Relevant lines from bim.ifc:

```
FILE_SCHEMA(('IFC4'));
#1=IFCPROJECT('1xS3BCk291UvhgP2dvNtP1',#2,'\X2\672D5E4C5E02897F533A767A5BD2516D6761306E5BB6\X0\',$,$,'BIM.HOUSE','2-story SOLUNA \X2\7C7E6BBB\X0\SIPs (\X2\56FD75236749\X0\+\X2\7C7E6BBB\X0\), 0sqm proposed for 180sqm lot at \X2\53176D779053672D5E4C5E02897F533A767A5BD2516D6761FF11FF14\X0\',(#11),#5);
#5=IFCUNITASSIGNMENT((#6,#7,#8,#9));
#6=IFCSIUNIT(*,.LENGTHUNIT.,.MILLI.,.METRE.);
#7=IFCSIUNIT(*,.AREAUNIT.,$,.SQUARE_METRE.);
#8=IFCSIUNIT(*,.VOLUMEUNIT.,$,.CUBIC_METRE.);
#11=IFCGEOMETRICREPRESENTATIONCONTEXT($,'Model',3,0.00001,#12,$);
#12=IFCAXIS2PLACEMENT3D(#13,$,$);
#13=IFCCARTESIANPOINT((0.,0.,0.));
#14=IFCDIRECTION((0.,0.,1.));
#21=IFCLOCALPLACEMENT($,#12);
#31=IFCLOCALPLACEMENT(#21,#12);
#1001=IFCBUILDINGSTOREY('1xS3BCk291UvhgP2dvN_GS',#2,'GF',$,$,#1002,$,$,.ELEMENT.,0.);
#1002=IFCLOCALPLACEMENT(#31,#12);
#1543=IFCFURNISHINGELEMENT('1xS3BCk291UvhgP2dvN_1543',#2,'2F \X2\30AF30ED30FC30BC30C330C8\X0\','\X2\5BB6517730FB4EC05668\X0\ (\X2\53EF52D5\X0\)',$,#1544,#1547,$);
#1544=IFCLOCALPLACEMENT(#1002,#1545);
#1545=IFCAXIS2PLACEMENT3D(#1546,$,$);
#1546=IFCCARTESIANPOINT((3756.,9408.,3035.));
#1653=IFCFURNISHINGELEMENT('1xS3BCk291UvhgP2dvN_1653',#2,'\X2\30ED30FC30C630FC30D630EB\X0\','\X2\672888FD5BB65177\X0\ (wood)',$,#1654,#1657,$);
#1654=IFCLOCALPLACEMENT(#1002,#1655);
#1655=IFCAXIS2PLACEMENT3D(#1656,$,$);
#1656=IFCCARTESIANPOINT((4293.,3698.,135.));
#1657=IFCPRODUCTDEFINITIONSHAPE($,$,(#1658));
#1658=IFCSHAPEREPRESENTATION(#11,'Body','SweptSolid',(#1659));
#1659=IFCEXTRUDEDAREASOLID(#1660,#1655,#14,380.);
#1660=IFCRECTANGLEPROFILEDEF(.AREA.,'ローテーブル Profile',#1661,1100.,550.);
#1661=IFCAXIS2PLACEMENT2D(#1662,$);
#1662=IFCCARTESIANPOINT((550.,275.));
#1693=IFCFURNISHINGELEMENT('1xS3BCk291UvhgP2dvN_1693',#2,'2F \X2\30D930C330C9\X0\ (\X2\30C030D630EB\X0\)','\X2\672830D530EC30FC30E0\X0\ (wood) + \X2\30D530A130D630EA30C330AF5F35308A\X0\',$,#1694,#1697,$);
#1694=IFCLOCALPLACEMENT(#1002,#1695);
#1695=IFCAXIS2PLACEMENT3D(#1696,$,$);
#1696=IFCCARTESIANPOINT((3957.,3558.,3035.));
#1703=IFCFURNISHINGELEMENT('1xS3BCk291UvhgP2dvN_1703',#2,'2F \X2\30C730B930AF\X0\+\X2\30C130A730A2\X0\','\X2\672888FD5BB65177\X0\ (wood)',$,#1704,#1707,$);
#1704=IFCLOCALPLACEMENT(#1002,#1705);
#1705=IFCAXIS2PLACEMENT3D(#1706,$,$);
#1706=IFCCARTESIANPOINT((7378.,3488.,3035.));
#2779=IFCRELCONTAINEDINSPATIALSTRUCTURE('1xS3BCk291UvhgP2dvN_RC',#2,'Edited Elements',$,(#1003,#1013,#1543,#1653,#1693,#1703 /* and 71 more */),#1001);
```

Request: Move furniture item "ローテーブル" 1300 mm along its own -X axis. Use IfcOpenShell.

```python
import ifcopenshell
import ifcopenshell.api.geometry
import ifcopenshell.util.placement
import ifcopenshell.util.unit

model = ifcopenshell.open("bim.ifc")
unit_scale = ifcopenshell.util.unit.calculate_unit_scale(model)

item = model.by_id(1653)
matrix = ifcopenshell.util.placement.get_local_placement(item.ObjectPlacement)
matrix[:3, 3] -= matrix[:3, 0] * 1.3 / unit_scale
ifcopenshell.api.geometry.edit_object_placement(model, product=item, matrix=matrix, is_si=False)

print(ifcopenshell.util.placement.get_local_placement(item.ObjectPlacement).round(3) + 0.0)

model.write("bim_updated.ifc")
```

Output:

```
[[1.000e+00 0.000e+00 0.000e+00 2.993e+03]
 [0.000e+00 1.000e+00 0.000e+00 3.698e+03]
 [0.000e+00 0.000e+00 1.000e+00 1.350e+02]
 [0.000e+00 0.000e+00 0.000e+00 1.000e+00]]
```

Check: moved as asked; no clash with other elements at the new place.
